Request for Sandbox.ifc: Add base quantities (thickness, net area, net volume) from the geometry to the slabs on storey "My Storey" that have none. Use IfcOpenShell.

First a look at what the model holds.

```python
import ifcopenshell
import ifcopenshell.util.element
import ifcopenshell.util.unit

model = ifcopenshell.open("Sandbox.ifc")
print(model.schema)
for unit_type in ("LENGTHUNIT", "AREAUNIT", "VOLUMEUNIT"):
    print(unit_type, ifcopenshell.util.unit.calculate_unit_scale(model, unit_type))
storey = next(s for s in model.by_type("IfcBuildingStorey") if s.Name == "My Storey")
slabs = [e for e in ifcopenshell.util.element.get_decomposition(storey) if e.is_a("IfcSlab")]
for e in sorted(slabs, key=lambda e: e.id()):
    print(e.id(), e.is_a(), e.Name, list(ifcopenshell.util.element.get_psets(e, qtos_only=True)), sep=" | ")
```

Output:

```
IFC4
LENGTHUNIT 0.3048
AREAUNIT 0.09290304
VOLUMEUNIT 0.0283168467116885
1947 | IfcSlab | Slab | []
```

```python
import ifcopenshell
import ifcopenshell.api.pset
import ifcopenshell.geom
import ifcopenshell.util.element
import ifcopenshell.util.shape
import ifcopenshell.util.unit

model = ifcopenshell.open("Sandbox.ifc")
unit_scale = ifcopenshell.util.unit.calculate_unit_scale(model)
area_scale = ifcopenshell.util.unit.calculate_unit_scale(model, "AREAUNIT")
volume_scale = ifcopenshell.util.unit.calculate_unit_scale(model, "VOLUMEUNIT")
settings = ifcopenshell.geom.settings()

storey = next(s for s in model.by_type("IfcBuildingStorey") if s.Name == "My Storey")
slabs = [e for e in ifcopenshell.util.element.get_decomposition(storey) if e.is_a("IfcSlab")]

for e in sorted(slabs, key=lambda e: e.id()):
    if ifcopenshell.util.element.get_psets(e, qtos_only=True, should_inherit=False):
        continue
    # Geometry comes back in metres, in the element's own axes.
    shape = ifcopenshell.geom.create_shape(settings, e)
    values = {
        "Width": ifcopenshell.util.shape.get_z(shape.geometry) / unit_scale,
        "NetArea": ifcopenshell.util.shape.get_footprint_area(shape.geometry) / area_scale,
        "NetVolume": ifcopenshell.util.shape.get_volume(shape.geometry) / volume_scale,
    }
    qto = ifcopenshell.api.pset.add_qto(model, product=e, name="Qto_SlabBaseQuantities")
    ifcopenshell.api.pset.edit_qto(model, qto=qto, properties=values)
    print(e.id(), {k: round(v, 3) for k, v in values.items()})

model.write("Sandbox_v2.ifc")
```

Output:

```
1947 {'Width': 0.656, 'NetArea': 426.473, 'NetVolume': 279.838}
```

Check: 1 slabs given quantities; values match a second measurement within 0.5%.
